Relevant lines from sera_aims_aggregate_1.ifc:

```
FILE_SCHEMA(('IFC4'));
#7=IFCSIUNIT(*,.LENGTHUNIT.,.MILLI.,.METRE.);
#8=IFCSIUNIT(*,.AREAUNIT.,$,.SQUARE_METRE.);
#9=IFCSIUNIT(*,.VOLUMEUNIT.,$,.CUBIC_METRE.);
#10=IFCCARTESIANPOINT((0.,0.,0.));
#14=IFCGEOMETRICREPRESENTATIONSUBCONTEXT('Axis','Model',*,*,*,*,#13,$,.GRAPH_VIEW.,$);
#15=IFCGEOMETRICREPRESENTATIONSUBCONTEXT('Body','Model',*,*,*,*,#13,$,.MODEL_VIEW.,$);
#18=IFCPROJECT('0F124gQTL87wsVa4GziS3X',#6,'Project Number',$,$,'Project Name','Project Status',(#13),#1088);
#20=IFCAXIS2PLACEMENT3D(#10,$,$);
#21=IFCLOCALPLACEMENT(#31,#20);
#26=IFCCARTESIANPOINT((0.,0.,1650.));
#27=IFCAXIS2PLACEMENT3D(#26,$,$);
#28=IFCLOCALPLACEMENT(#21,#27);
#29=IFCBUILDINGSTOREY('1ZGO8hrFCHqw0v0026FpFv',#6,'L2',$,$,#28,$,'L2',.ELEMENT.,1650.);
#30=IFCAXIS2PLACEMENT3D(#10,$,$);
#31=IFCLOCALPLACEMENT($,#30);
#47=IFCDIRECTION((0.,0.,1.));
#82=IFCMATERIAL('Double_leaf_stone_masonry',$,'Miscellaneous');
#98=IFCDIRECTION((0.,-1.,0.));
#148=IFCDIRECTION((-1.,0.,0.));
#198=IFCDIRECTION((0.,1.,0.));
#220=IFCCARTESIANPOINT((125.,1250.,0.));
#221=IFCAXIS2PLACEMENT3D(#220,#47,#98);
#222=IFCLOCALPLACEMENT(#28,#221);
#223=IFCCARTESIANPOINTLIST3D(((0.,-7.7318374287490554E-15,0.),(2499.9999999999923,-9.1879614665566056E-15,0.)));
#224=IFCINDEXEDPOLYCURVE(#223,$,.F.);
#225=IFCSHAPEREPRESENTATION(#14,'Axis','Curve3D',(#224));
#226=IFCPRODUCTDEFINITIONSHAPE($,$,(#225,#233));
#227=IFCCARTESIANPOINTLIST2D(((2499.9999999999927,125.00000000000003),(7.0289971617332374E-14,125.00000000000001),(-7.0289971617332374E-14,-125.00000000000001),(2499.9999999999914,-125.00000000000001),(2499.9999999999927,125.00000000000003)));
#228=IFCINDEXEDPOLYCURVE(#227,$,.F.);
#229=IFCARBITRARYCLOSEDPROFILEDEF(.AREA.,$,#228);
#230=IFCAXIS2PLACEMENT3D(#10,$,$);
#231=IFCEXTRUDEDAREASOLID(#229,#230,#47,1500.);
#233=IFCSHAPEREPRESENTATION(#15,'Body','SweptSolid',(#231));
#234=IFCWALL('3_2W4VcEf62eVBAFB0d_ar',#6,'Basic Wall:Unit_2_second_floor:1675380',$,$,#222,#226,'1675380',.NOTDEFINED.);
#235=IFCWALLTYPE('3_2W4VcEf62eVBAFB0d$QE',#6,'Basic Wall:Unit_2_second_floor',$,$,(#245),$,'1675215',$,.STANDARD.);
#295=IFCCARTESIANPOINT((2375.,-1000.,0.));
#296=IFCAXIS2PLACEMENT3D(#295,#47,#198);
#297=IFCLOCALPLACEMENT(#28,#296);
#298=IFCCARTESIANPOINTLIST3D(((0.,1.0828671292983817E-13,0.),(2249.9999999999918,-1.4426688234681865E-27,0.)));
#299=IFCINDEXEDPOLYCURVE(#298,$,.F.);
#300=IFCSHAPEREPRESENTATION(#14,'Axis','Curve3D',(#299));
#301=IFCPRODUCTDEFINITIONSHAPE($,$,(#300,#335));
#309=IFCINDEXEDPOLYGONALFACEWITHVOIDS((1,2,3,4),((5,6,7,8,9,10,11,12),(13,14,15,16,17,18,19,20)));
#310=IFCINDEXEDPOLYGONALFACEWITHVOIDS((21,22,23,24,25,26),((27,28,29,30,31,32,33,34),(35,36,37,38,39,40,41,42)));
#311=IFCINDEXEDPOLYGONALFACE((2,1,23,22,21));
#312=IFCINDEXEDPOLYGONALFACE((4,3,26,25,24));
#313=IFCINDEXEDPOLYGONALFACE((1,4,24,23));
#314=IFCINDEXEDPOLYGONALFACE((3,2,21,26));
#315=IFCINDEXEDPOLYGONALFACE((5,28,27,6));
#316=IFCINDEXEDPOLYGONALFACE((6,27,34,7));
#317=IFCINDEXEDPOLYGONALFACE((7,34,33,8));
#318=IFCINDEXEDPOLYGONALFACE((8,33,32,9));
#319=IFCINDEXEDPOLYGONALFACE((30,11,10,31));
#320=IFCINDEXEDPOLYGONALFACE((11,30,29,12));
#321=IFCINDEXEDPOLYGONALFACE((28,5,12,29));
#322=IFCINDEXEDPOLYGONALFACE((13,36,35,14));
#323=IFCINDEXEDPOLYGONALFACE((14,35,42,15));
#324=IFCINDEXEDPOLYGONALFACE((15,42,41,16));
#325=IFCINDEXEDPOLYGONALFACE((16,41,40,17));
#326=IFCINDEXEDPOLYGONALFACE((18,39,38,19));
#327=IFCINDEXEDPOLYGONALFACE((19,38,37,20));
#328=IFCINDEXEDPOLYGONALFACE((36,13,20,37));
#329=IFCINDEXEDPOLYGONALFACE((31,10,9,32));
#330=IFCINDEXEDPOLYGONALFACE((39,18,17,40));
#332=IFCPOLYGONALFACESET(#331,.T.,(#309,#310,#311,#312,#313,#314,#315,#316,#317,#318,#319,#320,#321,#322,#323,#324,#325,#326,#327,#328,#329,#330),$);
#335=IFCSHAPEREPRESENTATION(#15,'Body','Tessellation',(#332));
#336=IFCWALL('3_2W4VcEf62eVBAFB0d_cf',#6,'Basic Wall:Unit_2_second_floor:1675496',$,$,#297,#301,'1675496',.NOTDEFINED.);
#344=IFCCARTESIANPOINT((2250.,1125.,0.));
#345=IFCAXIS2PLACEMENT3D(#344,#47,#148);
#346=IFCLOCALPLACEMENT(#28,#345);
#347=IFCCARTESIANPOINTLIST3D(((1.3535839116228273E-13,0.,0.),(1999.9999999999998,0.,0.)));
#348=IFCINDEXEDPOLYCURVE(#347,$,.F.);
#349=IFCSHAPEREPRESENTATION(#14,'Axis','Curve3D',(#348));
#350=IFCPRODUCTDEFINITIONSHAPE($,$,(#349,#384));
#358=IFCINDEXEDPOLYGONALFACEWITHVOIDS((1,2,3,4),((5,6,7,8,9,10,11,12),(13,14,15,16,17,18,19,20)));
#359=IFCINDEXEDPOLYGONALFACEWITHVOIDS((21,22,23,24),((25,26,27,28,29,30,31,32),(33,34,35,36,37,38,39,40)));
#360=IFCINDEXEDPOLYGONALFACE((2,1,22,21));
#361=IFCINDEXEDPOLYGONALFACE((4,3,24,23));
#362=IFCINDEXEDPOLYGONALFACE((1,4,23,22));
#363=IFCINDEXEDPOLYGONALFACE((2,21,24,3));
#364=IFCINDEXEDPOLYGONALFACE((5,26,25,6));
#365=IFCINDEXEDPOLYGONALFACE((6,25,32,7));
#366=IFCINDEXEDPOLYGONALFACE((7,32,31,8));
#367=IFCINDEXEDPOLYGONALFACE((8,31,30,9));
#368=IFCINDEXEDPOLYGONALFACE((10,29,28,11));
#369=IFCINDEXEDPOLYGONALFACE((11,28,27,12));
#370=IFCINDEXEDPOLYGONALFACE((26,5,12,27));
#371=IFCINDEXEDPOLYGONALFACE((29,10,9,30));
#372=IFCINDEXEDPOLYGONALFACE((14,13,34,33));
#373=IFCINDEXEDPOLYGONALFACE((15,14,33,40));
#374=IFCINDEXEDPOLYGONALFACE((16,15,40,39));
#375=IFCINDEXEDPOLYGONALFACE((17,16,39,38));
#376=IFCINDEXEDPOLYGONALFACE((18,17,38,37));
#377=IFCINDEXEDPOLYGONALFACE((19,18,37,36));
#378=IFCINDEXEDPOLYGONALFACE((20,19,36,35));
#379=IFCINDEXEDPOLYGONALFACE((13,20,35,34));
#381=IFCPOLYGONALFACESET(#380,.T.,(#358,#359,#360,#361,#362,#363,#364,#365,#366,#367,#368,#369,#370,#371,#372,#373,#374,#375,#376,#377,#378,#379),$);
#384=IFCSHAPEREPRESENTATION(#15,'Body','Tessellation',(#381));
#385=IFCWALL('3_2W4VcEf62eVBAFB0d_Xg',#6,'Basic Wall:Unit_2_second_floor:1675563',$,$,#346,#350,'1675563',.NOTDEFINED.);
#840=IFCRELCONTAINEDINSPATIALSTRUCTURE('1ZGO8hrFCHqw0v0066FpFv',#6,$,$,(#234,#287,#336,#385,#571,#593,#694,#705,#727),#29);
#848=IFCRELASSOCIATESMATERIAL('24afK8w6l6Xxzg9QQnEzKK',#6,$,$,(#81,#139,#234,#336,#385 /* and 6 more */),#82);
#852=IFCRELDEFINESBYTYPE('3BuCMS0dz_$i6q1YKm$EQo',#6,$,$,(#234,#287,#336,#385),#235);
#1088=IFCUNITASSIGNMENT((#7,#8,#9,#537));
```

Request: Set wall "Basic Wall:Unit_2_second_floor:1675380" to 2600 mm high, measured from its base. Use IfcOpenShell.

```python
import ifcopenshell
import ifcopenshell.geom
import ifcopenshell.util.representation
import ifcopenshell.util.shape

model = ifcopenshell.open("sera_aims_aggregate_1.ifc")
settings = ifcopenshell.geom.settings()


def volume(element):
    """Net volume in cubic metres, openings subtracted."""
    shape = ifcopenshell.geom.create_shape(settings, element)
    return ifcopenshell.util.shape.get_volume(shape.geometry)


wall = model.by_guid("3_2W4VcEf62eVBAFB0d_ar")
before = volume(wall)

body = ifcopenshell.util.representation.get_representation(wall, "Model", "Body")
solid = body.Items[0]
old_height = solid.Depth
solid.Depth = 2600.0
after = volume(wall)

print(f"height {old_height:g} -> {solid.Depth:g}, volume {before:.3f} -> {after:.3f} m3")

model.write("sera_aims_aggregate_1_updated.ifc")
```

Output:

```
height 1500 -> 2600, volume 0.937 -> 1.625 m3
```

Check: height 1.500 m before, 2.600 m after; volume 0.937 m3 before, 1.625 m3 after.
